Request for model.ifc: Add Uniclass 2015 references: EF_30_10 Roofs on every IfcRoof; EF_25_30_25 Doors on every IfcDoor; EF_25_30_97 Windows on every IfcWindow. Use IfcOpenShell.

First a look at what the model holds.

```python
import ifcopenshell

model = ifcopenshell.open("model.ifc")
print(model.schema)
print("classifications:", [c.Name for c in model.by_type("IfcClassification")])
for ifc_class in ("IfcDoor", "IfcRoof", "IfcStair", "IfcWall", "IfcWindow"):
    print(ifc_class, len(model.by_type(ifc_class)))
```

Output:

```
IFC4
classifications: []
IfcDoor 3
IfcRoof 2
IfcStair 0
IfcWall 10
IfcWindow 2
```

```python
import ifcopenshell
import ifcopenshell.api.classification

model = ifcopenshell.open("model.ifc")

system = ifcopenshell.api.classification.add_classification(model, classification="Uniclass 2015")

codes = {
    "IfcRoof": ("EF_30_10", "Roofs"),
    "IfcDoor": ("EF_25_30_25", "Doors"),
    "IfcWindow": ("EF_25_30_97", "Windows"),
}
for ifc_class, (code, name) in codes.items():
    products = model.by_type(ifc_class)
    ifcopenshell.api.classification.add_reference(
        model, products=products, classification=system, identification=code, name=name
    )
    print(code, len(products))

model.write("model_rev.ifc")
```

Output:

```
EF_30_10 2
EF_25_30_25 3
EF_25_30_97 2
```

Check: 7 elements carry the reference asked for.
